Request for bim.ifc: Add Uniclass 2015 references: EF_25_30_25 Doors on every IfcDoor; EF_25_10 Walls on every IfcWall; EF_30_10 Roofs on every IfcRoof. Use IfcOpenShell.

First a look at what the model holds.

```python
import ifcopenshell

model = ifcopenshell.open("bim.ifc")
print(model.schema)
print("classifications:", [c.Name for c in model.by_type("IfcClassification")])
for ifc_class in ("IfcDoor", "IfcRoof", "IfcStair", "IfcWall", "IfcWindow"):
    print(ifc_class, len(model.by_type(ifc_class)))
```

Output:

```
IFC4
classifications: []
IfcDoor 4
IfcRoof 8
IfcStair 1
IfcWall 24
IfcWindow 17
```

```python
import ifcopenshell
import ifcopenshell.api.classification

model = ifcopenshell.open("bim.ifc")

system = ifcopenshell.api.classification.add_classification(model, classification="Uniclass 2015")

codes = {
    "IfcDoor": ("EF_25_30_25", "Doors"),
    "IfcWall": ("EF_25_10", "Walls"),
    "IfcRoof": ("EF_30_10", "Roofs"),
}
for ifc_class, (code, name) in codes.items():
    products = model.by_type(ifc_class)
    ifcopenshell.api.classification.add_reference(
        model, products=products, classification=system, identification=code, name=name
    )
    print(code, len(products))

model.write("bim_edited.ifc")
```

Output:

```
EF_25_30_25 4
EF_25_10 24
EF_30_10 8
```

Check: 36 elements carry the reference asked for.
